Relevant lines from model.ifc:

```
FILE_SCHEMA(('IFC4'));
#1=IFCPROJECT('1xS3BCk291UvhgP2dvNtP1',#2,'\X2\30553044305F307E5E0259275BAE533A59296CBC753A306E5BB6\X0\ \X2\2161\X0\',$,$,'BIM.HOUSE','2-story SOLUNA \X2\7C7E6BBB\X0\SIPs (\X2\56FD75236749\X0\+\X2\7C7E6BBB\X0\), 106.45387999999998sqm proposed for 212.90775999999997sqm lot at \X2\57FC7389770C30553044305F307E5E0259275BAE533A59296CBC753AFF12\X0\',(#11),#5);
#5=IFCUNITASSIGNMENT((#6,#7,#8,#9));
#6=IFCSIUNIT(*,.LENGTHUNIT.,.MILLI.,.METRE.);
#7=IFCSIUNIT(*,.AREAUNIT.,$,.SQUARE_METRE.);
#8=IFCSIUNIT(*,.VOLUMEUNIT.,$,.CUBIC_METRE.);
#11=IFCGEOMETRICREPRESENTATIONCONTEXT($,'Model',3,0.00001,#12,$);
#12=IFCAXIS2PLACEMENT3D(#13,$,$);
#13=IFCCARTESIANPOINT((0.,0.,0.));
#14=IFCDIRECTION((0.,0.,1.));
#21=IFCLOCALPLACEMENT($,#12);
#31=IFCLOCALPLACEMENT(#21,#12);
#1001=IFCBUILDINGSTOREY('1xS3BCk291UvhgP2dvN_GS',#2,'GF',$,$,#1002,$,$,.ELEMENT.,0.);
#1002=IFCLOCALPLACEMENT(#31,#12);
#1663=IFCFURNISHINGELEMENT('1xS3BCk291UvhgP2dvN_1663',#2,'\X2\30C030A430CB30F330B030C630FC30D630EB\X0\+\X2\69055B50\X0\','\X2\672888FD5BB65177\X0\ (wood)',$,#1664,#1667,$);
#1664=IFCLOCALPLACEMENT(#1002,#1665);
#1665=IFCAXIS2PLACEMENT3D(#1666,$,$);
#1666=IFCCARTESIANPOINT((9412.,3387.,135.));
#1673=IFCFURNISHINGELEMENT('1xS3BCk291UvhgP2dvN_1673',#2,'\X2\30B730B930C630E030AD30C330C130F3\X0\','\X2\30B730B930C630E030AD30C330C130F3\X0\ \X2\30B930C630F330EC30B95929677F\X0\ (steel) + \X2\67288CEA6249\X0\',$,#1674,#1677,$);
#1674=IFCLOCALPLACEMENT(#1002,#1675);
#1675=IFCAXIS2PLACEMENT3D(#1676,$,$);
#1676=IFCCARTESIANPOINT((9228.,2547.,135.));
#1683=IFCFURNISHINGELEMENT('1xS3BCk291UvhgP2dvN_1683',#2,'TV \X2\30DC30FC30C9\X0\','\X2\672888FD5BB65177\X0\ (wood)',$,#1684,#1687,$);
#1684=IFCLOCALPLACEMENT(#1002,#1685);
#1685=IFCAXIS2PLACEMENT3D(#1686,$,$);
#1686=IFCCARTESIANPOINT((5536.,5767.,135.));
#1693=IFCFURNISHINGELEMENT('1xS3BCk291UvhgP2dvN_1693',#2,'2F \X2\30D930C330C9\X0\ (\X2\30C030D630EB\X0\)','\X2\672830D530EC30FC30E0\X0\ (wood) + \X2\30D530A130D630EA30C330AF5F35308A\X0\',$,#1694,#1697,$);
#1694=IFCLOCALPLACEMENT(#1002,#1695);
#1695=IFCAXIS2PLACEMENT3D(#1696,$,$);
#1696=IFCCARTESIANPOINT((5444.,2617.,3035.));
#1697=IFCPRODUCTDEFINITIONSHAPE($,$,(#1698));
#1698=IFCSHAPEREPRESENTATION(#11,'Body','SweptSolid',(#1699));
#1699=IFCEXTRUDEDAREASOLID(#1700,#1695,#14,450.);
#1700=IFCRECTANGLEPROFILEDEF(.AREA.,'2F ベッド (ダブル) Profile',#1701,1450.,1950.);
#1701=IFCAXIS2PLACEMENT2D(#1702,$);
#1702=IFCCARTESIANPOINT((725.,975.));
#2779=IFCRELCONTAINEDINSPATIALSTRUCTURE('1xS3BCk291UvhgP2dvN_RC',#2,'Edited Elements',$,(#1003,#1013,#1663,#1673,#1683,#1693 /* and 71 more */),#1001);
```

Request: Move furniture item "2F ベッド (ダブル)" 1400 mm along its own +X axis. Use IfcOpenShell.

```python
import ifcopenshell
import ifcopenshell.api.geometry
import ifcopenshell.util.placement
import ifcopenshell.util.unit

model = ifcopenshell.open("model.ifc")
unit_scale = ifcopenshell.util.unit.calculate_unit_scale(model)

item = model.by_id(1693)
matrix = ifcopenshell.util.placement.get_local_placement(item.ObjectPlacement)
matrix[:3, 3] += matrix[:3, 0] * 1.4 / unit_scale
ifcopenshell.api.geometry.edit_object_placement(model, product=item, matrix=matrix, is_si=False)

print(ifcopenshell.util.placement.get_local_placement(item.ObjectPlacement).round(3) + 0.0)

model.write("model_rev.ifc")
```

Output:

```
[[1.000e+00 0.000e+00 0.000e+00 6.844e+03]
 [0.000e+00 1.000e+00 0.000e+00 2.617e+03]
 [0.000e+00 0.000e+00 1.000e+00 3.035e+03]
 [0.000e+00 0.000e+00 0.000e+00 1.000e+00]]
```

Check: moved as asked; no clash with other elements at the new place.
